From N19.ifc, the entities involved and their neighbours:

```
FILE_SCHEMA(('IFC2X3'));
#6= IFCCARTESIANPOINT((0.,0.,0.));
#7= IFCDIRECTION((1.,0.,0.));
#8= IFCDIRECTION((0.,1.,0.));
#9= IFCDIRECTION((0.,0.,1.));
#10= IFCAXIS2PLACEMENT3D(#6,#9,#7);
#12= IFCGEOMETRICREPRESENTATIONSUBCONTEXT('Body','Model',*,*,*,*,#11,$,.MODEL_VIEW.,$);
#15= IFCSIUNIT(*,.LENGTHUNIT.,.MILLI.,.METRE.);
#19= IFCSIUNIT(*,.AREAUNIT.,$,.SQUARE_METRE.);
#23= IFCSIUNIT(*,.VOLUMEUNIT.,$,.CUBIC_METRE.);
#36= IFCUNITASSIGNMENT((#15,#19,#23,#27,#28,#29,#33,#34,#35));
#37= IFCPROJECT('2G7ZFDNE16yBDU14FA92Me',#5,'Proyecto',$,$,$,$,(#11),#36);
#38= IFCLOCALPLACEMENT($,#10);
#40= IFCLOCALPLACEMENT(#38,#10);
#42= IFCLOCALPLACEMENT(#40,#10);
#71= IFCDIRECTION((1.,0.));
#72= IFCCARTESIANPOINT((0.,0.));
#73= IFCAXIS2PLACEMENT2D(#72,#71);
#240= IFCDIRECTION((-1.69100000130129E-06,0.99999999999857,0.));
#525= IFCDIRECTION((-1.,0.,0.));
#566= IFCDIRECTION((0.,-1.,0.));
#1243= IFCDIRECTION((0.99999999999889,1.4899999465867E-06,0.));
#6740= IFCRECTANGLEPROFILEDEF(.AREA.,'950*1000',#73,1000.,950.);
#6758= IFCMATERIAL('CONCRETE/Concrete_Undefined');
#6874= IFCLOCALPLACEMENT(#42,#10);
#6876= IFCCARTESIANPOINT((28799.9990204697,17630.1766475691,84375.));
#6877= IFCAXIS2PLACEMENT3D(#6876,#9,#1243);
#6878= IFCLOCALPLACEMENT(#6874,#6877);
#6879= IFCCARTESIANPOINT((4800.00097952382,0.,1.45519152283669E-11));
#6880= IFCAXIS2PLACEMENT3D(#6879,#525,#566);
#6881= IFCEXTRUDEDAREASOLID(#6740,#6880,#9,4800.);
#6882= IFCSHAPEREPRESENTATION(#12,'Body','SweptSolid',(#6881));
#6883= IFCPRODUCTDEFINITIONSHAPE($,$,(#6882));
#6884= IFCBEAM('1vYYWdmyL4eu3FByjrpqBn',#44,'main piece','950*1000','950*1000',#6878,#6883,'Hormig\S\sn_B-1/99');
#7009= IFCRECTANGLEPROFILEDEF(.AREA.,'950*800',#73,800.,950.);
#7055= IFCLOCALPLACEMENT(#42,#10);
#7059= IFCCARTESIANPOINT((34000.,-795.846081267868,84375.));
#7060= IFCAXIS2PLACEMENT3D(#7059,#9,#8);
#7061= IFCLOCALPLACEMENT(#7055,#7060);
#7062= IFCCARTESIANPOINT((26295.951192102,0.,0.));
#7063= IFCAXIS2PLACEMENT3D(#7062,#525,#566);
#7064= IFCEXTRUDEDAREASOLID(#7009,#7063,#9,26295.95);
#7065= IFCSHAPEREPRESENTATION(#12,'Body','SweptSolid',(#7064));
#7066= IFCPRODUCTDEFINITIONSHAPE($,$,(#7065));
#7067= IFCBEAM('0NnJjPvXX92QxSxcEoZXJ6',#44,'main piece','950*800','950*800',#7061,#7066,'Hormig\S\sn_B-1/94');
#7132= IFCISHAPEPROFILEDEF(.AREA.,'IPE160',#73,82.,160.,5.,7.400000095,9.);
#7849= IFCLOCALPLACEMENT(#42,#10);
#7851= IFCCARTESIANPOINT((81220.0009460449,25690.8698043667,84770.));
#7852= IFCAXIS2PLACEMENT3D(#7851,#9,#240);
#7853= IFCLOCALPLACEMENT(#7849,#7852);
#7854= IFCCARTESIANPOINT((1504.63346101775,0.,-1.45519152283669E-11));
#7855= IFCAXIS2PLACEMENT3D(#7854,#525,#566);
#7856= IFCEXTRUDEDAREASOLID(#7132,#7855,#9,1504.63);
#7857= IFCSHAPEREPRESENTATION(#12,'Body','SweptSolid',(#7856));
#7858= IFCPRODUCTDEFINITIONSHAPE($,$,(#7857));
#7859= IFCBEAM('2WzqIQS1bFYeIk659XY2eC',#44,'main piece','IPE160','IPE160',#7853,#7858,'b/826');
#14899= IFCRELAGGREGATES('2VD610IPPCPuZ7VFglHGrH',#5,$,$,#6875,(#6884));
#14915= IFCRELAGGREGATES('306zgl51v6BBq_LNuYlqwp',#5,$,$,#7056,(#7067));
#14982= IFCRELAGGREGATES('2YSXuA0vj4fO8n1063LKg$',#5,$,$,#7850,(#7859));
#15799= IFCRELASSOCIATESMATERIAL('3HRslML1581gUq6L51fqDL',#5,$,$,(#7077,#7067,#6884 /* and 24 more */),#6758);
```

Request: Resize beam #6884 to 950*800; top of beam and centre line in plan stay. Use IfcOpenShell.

```python
import ifcopenshell
import ifcopenshell.util.element
import ifcopenshell.util.representation

model = ifcopenshell.open("N19.ifc")

member = model.by_id(6884)
source = next(p for p in model.by_type("IfcRectangleProfileDef") if p.ProfileName == "950*800")

body = ifcopenshell.util.representation.get_representation(member, "Model", "Body")
solid = body.Items[0]
old_profile = solid.SweptArea

# Copy the section's sizes but keep this member's own profile position.
profile = ifcopenshell.util.element.copy(model, source)
# Profiles are centred, so shift by half the change in depth to hold the top.
shift = (old_profile.YDim - profile.YDim) / 2
x, y = old_profile.Position.Location.Coordinates
up = (0.0, 1.0)  # upwards, in the solid's own plane
location = model.createIfcCartesianPoint((x + up[0] * shift, y + up[1] * shift))
profile.Position = model.createIfcAxis2Placement2D(location, old_profile.Position.RefDirection)
solid.SweptArea = profile
if not model.get_total_inverses(old_profile):
    ifcopenshell.util.element.remove_deep2(model, old_profile)
member.Description = member.Description.replace("950*1000", "950*800")
member.ObjectType = member.ObjectType.replace("950*1000", "950*800")

print(solid.SweptArea)

model.write("N19_v2.ifc")
```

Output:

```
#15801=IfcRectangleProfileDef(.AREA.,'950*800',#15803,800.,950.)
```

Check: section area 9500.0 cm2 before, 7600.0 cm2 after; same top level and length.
